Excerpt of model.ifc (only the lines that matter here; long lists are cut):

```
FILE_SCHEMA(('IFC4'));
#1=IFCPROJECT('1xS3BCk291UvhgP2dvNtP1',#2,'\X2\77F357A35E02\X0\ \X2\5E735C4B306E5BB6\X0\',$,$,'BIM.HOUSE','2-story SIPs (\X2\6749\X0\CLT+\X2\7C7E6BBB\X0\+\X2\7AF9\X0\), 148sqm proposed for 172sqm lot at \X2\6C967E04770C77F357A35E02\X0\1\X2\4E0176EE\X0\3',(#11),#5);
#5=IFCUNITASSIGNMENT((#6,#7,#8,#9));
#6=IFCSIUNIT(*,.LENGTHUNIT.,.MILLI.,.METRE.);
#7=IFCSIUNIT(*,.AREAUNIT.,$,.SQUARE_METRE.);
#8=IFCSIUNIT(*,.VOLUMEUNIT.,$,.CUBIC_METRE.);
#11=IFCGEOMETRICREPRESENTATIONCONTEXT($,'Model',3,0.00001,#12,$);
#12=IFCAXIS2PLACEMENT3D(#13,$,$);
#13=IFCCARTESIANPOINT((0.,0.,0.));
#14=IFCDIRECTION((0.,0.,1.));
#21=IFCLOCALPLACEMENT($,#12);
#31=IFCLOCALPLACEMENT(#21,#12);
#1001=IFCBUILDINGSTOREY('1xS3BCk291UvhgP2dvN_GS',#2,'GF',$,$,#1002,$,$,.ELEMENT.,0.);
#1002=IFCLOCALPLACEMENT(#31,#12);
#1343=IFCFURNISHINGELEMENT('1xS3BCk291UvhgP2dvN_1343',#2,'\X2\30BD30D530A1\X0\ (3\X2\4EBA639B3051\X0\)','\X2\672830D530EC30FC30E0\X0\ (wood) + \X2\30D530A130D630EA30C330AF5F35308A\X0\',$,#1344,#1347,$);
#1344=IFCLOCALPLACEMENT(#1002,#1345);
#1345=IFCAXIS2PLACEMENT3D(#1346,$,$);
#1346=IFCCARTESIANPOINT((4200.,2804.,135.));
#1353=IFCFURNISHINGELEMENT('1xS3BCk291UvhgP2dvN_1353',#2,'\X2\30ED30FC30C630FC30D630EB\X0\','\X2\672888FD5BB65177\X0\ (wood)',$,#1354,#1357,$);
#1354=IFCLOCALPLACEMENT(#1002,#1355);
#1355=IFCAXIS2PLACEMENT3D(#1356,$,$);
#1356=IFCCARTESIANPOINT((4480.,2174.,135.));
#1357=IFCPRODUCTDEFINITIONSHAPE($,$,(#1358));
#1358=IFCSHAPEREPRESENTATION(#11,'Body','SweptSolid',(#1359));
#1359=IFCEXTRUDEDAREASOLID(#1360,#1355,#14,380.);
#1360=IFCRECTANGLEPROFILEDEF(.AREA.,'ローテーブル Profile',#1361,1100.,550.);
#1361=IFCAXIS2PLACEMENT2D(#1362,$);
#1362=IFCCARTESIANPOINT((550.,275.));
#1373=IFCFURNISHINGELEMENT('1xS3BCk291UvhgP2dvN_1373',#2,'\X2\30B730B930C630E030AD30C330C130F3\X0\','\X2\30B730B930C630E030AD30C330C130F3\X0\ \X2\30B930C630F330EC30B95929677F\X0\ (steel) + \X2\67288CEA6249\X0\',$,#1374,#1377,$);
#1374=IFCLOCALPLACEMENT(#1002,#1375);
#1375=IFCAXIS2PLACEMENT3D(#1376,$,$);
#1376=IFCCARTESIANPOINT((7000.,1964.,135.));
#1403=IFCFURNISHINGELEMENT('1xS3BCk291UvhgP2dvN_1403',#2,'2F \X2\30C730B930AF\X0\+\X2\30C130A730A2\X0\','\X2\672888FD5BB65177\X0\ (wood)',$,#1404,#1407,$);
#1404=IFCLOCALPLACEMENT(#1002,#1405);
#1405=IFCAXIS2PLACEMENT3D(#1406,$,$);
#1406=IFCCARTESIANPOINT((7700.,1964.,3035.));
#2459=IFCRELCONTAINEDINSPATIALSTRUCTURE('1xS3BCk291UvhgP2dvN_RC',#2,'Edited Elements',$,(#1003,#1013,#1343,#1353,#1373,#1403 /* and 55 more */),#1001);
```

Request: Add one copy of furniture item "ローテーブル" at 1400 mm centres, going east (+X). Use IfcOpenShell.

```python
import numpy as np
import ifcopenshell
import ifcopenshell.api.geometry
import ifcopenshell.api.root
import ifcopenshell.util.element
import ifcopenshell.util.placement

model = ifcopenshell.open("model.ifc")


def reuse_history(source, copy):
    """copy_class also copies each property set's owner history, people and application; keep the originals."""
    for rel in copy.IsDefinedBy:
        if rel.is_a("IfcRelDefinesByProperties") and (history := rel.RelatingPropertyDefinition.OwnerHistory):
            rel.RelatingPropertyDefinition.OwnerHistory = source.OwnerHistory
            ifcopenshell.util.element.remove_deep2(model, history)


source = model.by_guid("1xS3BCk291UvhgP2dvN_1353")
base = ifcopenshell.util.placement.get_local_placement(source.ObjectPlacement)
step = np.array([1.0, 0.0, 0.0]) * 1400.0

for i in range(1, 2):
    copy = ifcopenshell.api.root.copy_class(model, product=source)
    copy.Representation = ifcopenshell.util.element.copy_deep(
        model, source.Representation, exclude=["IfcGeometricRepresentationContext", "IfcRepresentationMap"]
    )
    reuse_history(source, copy)
    matrix = base.copy()
    matrix[:3, 3] += i * step
    print("added at", matrix[:3, 3].round(3) + 0.0)
    ifcopenshell.api.geometry.edit_object_placement(model, product=copy, matrix=matrix, is_si=False)

model.write("model_v2.ifc")
```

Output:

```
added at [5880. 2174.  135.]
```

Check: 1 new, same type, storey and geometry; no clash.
